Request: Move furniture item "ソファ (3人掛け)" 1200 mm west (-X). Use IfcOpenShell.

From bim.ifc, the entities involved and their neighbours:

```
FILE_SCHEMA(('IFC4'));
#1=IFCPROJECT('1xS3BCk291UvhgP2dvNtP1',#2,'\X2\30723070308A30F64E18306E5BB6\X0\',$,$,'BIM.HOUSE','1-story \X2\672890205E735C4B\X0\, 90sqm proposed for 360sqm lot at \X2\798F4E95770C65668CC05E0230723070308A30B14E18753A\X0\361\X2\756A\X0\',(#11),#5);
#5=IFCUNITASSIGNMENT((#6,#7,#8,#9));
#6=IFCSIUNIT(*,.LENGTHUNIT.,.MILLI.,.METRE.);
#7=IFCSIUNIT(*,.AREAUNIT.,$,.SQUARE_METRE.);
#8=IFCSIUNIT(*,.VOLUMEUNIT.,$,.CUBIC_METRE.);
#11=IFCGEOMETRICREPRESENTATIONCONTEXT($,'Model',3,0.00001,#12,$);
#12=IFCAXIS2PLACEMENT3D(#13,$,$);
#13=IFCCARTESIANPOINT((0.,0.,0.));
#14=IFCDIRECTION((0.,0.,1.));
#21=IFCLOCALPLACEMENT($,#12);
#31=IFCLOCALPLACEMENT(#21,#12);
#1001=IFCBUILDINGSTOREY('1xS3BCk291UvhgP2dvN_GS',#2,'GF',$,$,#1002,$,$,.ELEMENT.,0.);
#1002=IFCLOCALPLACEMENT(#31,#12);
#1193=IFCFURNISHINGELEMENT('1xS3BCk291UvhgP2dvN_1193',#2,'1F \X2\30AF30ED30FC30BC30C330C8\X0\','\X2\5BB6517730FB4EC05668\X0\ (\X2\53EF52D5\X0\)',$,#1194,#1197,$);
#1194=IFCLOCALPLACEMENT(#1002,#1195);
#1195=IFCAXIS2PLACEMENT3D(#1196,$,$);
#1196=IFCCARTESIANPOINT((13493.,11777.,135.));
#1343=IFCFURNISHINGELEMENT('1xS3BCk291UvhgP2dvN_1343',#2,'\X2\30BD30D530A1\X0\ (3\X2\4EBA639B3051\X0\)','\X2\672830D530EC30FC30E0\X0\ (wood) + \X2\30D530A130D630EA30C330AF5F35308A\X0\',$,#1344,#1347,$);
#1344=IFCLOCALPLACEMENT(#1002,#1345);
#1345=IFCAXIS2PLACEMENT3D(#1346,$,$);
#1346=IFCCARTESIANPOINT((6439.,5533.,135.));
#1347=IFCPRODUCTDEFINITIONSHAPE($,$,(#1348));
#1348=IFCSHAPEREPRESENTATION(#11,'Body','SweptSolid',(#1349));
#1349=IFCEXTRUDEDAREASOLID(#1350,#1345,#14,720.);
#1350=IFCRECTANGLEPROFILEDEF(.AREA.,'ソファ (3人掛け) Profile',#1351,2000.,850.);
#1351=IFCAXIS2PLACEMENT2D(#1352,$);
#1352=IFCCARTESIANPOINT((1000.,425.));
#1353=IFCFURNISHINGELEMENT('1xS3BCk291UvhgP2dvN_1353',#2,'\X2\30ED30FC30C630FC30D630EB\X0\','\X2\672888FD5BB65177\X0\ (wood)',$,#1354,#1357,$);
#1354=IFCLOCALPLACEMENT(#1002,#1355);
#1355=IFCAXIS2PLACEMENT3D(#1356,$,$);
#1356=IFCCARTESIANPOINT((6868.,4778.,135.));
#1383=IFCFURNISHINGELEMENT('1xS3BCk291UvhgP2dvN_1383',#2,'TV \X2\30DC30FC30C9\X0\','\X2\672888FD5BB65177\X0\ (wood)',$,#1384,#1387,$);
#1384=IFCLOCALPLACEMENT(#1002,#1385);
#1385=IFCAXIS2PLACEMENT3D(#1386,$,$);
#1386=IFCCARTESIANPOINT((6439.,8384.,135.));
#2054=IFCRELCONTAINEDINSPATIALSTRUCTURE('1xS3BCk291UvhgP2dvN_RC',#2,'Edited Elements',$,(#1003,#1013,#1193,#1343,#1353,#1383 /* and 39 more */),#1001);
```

```python
import ifcopenshell
import ifcopenshell.api.geometry
import ifcopenshell.util.placement
import ifcopenshell.util.unit

model = ifcopenshell.open("bim.ifc")
unit_scale = ifcopenshell.util.unit.calculate_unit_scale(model)

item = model.by_id(1343)
matrix = ifcopenshell.util.placement.get_local_placement(item.ObjectPlacement)
matrix[0, 3] -= 1.2 / unit_scale
ifcopenshell.api.geometry.edit_object_placement(model, product=item, matrix=matrix, is_si=False)

print(ifcopenshell.util.placement.get_local_placement(item.ObjectPlacement).round(3) + 0.0)

model.write("bim-out.ifc")
```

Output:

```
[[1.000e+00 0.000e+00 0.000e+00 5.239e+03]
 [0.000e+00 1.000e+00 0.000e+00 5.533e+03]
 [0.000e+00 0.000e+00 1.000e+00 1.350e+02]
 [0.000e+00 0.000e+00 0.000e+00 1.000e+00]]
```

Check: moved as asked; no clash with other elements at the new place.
